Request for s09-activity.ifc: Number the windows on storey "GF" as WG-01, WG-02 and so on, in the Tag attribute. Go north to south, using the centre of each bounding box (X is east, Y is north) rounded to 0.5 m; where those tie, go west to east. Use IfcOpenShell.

First a look at what the model holds.

```python
import ifcopenshell
import ifcopenshell.util.element
import ifcopenshell.util.placement

model = ifcopenshell.open("s09-activity.ifc")
print(model.schema)
storey = next(s for s in model.by_type("IfcBuildingStorey") if s.Name == "GF")
windows = [e for e in ifcopenshell.util.element.get_decomposition(storey) if e.is_a("IfcWindow")]
for e in sorted(windows, key=lambda e: e.id()):
    origin = ifcopenshell.util.placement.get_local_placement(e.ObjectPlacement)[:3, 3]
    print(e.id(), e.Tag, e.Name, origin.round(2) + 0.0, sep=" | ")
```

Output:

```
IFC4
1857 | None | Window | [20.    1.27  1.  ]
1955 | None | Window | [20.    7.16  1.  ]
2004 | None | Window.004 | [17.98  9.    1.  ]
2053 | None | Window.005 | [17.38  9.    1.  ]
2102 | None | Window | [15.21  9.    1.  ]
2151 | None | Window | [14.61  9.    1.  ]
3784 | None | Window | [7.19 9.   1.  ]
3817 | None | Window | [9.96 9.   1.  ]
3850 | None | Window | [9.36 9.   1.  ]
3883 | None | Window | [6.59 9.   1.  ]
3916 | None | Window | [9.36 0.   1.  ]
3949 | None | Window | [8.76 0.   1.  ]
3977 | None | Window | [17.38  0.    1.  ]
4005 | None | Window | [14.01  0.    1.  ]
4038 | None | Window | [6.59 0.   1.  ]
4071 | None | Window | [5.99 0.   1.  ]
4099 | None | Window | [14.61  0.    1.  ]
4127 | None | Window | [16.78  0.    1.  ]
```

```python
import ifcopenshell
import ifcopenshell.geom
import ifcopenshell.util.element
import ifcopenshell.util.shape

model = ifcopenshell.open("s09-activity.ifc")
settings = ifcopenshell.geom.settings()
settings.set("use-world-coords", True)


def centre(element):
    shape = ifcopenshell.geom.create_shape(settings, element)
    return ifcopenshell.util.shape.get_bbox_centroid(shape.geometry)


storey = next(s for s in model.by_type("IfcBuildingStorey") if s.Name == "GF")
windows = [e for e in ifcopenshell.util.element.get_decomposition(storey) if e.is_a("IfcWindow")]

# Insertion points can sit at a corner or the storey origin, so sort by the geometry (in metres).
centres = {e: centre(e) for e in windows}
windows.sort(key=lambda e: (-round(centres[e][1] / 0.5), centres[e][0]))

for i, e in enumerate(windows, start=1):
    number = f"WG-{i:02d}"
    e.Tag = number
    print(e.id(), number)

model.write("s09-activity_v2.ifc")
```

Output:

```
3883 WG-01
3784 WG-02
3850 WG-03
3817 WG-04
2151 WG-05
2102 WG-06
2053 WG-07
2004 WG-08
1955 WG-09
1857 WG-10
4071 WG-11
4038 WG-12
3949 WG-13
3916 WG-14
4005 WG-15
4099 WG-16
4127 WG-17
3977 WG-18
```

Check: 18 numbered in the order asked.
